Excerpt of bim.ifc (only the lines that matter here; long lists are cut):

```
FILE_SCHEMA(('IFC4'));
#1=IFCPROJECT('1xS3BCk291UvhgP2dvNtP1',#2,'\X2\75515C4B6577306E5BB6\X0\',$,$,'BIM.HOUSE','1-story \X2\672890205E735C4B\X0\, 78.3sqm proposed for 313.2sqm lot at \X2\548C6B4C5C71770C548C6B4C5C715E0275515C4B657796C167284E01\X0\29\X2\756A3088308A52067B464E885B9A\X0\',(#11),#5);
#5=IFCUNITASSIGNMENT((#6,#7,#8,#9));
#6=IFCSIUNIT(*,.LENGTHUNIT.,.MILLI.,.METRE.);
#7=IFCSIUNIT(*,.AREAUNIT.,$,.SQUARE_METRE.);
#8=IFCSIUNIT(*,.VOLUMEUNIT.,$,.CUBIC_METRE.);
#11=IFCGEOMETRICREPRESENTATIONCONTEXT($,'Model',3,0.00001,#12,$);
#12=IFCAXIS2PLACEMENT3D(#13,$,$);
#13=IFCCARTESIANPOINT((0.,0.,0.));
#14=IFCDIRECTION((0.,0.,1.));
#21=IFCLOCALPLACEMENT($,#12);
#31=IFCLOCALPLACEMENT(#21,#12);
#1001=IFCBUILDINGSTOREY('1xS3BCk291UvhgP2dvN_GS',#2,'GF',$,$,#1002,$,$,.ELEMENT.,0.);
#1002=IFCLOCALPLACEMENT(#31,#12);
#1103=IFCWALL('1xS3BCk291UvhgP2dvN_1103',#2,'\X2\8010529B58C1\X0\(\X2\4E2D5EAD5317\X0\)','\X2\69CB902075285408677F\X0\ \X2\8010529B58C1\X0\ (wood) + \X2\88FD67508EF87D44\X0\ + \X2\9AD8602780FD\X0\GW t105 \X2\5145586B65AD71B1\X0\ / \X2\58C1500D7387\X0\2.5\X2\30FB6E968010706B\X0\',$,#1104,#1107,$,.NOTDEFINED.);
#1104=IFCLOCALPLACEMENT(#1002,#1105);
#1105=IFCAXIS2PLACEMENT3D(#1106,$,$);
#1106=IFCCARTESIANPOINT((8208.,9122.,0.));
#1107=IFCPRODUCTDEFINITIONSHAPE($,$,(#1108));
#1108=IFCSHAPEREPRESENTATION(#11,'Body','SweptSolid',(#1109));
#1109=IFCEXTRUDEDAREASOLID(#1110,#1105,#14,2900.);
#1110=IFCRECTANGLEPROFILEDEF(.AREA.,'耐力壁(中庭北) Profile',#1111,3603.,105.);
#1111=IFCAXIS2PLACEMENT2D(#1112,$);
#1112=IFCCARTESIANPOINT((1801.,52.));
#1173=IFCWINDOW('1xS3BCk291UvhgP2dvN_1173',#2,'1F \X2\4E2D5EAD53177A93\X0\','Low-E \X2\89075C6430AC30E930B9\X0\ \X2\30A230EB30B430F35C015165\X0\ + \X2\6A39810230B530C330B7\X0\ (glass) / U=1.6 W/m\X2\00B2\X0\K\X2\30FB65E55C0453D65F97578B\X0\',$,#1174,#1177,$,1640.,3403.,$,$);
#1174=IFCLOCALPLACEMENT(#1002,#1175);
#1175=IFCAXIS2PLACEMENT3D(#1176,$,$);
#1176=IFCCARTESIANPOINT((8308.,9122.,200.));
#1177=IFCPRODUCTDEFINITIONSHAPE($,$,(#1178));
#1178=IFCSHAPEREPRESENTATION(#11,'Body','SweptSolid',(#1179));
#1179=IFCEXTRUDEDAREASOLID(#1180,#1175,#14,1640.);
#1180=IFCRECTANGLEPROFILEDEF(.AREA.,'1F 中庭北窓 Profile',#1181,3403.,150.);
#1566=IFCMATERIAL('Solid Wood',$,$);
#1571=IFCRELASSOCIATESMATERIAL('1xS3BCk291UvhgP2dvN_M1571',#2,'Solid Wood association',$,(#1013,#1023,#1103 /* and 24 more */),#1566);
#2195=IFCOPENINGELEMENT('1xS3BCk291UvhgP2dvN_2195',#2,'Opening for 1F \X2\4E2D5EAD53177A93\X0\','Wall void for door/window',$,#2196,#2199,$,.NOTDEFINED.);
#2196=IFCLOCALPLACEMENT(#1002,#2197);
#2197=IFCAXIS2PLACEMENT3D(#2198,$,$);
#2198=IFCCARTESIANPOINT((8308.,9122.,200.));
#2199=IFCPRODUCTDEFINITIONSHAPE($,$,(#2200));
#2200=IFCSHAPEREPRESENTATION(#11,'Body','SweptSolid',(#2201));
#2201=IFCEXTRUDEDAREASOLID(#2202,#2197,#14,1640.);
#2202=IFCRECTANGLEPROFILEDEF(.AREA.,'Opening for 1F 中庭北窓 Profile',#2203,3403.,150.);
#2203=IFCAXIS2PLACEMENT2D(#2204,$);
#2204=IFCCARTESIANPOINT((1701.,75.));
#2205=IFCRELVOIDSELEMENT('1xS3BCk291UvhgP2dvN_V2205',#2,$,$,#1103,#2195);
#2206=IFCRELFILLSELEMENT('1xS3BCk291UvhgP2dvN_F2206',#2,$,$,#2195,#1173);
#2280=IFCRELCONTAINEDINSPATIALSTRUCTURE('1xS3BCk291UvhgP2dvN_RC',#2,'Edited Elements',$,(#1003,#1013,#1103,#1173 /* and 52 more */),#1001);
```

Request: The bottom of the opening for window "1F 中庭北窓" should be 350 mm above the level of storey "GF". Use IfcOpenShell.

```python
import numpy as np
import ifcopenshell
import ifcopenshell.api.geometry
import ifcopenshell.geom
import ifcopenshell.util.element
import ifcopenshell.util.placement
import ifcopenshell.util.shape
import ifcopenshell.util.unit

model = ifcopenshell.open("bim.ifc")
unit_scale = ifcopenshell.util.unit.calculate_unit_scale(model)

window = model.by_guid("1xS3BCk291UvhgP2dvN_1173")
opening = window.FillsVoids[0].RelatingOpeningElement
storey = ifcopenshell.util.element.get_container(window, ifc_class="IfcBuildingStorey")
level = ifcopenshell.util.placement.get_local_placement(storey.ObjectPlacement)[2, 3]

# The opening's origin need not be at the sill, so measure its lowest point.
shape = ifcopenshell.geom.create_shape(ifcopenshell.geom.settings(), opening)
bottom = ifcopenshell.util.shape.get_shape_bottom_elevation(shape, shape.geometry) / unit_scale
dz = level + 0.35 / unit_scale - bottom

shift = np.array([0.0, 0.0, dz])
# The window is not placed relative to its opening, so move both.
for product in (opening, window):
    matrix = ifcopenshell.util.placement.get_local_placement(product.ObjectPlacement)
    matrix[:3, 3] += shift
    ifcopenshell.api.geometry.edit_object_placement(model, product=product, matrix=matrix, is_si=False)

print(f"moved by {dz * unit_scale:+.3f} m")

model.write("bim_rev.ifc")
```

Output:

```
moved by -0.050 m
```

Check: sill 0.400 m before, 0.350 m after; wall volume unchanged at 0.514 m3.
